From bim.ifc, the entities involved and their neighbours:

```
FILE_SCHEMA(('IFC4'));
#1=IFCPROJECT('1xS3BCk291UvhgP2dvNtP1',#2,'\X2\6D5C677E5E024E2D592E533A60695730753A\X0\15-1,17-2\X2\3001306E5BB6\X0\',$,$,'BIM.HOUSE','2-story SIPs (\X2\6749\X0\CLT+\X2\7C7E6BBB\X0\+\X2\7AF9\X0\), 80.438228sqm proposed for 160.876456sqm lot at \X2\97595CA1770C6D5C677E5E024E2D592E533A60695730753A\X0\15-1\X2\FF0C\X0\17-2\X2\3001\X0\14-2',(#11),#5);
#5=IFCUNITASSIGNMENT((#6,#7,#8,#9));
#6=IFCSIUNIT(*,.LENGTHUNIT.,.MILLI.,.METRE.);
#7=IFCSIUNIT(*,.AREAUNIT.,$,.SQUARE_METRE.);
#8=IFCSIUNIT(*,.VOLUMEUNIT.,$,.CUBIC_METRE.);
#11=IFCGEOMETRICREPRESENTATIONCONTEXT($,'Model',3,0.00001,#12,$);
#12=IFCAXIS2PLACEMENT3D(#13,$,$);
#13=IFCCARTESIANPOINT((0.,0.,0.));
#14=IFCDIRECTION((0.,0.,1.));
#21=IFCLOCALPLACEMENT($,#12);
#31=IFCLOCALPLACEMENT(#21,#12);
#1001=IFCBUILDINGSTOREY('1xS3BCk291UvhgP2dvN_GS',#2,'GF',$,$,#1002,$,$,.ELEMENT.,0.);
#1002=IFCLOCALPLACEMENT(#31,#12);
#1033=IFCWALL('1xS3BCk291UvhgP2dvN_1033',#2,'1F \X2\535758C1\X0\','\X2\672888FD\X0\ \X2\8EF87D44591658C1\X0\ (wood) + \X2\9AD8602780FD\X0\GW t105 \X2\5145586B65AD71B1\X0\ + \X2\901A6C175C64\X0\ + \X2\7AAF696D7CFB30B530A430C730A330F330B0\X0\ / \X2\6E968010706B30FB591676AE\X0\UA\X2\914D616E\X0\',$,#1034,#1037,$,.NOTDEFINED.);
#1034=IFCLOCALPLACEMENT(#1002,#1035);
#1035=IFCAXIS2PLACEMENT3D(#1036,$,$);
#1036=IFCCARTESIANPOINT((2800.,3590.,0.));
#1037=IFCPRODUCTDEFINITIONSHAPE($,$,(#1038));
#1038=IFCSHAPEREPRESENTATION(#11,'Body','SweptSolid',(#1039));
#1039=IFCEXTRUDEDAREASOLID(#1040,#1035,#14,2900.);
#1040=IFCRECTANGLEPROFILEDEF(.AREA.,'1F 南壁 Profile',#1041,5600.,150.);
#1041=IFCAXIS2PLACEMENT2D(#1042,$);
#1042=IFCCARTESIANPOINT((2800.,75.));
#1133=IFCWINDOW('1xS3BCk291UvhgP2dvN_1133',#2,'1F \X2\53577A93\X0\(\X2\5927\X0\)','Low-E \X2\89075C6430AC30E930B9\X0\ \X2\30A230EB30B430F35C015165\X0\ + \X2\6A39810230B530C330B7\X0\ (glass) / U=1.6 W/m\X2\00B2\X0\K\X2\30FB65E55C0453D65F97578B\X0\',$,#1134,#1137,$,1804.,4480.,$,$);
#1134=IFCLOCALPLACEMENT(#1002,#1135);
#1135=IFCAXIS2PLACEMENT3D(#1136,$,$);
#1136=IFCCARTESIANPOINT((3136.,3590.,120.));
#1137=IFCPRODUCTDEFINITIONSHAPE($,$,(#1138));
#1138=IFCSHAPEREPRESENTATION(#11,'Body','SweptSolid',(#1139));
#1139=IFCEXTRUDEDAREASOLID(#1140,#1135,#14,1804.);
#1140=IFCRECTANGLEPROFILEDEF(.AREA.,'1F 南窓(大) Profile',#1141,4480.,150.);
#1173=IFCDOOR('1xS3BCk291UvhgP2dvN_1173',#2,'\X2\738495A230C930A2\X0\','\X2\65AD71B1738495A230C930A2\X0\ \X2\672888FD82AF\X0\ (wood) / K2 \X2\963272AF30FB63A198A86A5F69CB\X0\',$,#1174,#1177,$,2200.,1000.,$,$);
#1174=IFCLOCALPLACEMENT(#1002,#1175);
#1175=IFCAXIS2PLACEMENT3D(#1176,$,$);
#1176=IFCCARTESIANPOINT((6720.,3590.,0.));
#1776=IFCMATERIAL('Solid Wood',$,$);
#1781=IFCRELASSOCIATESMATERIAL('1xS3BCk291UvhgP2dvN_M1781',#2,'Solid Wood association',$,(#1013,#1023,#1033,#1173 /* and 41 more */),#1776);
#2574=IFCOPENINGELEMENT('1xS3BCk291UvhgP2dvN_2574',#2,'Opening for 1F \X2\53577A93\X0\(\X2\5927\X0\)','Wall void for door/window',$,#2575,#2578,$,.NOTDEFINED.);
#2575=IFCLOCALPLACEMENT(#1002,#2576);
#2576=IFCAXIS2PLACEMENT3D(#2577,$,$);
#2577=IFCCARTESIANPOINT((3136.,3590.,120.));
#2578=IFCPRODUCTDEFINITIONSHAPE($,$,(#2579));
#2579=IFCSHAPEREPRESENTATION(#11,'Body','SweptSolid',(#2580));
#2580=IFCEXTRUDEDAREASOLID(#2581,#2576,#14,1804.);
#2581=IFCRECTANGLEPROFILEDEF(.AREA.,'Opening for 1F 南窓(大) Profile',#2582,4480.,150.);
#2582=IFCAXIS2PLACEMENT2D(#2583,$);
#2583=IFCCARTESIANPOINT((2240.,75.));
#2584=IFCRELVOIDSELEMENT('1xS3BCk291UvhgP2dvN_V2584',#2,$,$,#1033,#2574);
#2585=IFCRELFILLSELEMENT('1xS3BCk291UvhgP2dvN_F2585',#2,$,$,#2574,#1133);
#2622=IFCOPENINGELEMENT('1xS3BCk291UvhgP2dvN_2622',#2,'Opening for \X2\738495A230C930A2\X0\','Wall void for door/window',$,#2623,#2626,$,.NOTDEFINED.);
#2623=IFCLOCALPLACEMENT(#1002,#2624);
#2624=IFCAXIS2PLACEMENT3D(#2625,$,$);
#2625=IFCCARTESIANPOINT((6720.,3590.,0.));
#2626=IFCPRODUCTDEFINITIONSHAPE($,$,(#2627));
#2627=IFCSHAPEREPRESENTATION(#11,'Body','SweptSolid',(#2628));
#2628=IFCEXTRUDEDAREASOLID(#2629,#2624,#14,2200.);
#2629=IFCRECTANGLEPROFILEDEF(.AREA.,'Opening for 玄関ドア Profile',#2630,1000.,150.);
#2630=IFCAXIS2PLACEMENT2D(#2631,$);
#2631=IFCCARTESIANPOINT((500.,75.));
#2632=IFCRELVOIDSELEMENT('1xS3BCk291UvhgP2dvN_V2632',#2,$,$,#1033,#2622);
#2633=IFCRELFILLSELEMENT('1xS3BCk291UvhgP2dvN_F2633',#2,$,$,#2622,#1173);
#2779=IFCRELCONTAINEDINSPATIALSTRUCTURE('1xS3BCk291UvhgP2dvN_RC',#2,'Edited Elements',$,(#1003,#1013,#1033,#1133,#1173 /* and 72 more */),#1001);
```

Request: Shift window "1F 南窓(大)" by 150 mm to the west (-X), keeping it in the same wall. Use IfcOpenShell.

```python
import ifcopenshell
import ifcopenshell.api.geometry
import ifcopenshell.util.placement

model = ifcopenshell.open("bim.ifc")

window = model.by_guid("1xS3BCk291UvhgP2dvN_1133")
opening = window.FillsVoids[0].RelatingOpeningElement
wall = opening.VoidsElements[0].RelatingBuildingElement

wall_matrix = ifcopenshell.util.placement.get_local_placement(wall.ObjectPlacement)
shift = wall_matrix[:3, 0] * -150.0
before = ifcopenshell.util.placement.get_local_placement(window.ObjectPlacement)[:3, 3].copy()

# The window is not placed relative to its opening, so move both.
for product in (opening, window):
    matrix = ifcopenshell.util.placement.get_local_placement(product.ObjectPlacement)
    matrix[:3, 3] += shift
    ifcopenshell.api.geometry.edit_object_placement(model, product=product, matrix=matrix, is_si=False)

after = ifcopenshell.util.placement.get_local_placement(window.ObjectPlacement)[:3, 3]
print("window moved by", (after - before).round(3) + 0.0)

model.write("bim_updated.ifc")
```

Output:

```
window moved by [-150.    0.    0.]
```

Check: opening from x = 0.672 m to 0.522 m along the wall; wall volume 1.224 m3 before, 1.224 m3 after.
